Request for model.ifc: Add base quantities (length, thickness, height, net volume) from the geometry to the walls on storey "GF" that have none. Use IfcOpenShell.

First a look at what the model holds.

```python
import ifcopenshell
import ifcopenshell.util.element
import ifcopenshell.util.unit

model = ifcopenshell.open("model.ifc")
print(model.schema)
for unit_type in ("LENGTHUNIT", "AREAUNIT", "VOLUMEUNIT"):
    print(unit_type, ifcopenshell.util.unit.calculate_unit_scale(model, unit_type))
storey = next(s for s in model.by_type("IfcBuildingStorey") if s.Name == "GF")
walls = [e for e in ifcopenshell.util.element.get_decomposition(storey) if e.is_a("IfcWall")]
for e in sorted(walls, key=lambda e: e.id()):
    print(e.id(), e.is_a(), e.Name, list(ifcopenshell.util.element.get_psets(e, qtos_only=True)), sep=" | ")
```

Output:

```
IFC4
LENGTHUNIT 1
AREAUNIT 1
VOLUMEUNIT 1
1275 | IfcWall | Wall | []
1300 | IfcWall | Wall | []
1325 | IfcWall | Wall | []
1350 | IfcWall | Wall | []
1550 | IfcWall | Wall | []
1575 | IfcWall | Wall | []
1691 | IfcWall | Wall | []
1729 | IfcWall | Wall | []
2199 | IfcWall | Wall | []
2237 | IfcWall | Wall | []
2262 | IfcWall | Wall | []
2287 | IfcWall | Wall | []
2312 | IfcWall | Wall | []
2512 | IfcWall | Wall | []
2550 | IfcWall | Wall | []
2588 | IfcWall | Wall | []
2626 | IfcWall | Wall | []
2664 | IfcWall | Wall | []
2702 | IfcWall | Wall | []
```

```python
import ifcopenshell
import ifcopenshell.api.pset
import ifcopenshell.geom
import ifcopenshell.util.element
import ifcopenshell.util.shape
import ifcopenshell.util.unit

model = ifcopenshell.open("model.ifc")
unit_scale = ifcopenshell.util.unit.calculate_unit_scale(model)
volume_scale = ifcopenshell.util.unit.calculate_unit_scale(model, "VOLUMEUNIT")
settings = ifcopenshell.geom.settings()

storey = next(s for s in model.by_type("IfcBuildingStorey") if s.Name == "GF")
walls = [e for e in ifcopenshell.util.element.get_decomposition(storey) if e.is_a("IfcWall")]

for e in sorted(walls, key=lambda e: e.id()):
    if ifcopenshell.util.element.get_psets(e, qtos_only=True, should_inherit=False):
        continue
    # Geometry comes back in metres, in the element's own axes.
    shape = ifcopenshell.geom.create_shape(settings, e)
    values = {
        "Length": ifcopenshell.util.shape.get_x(shape.geometry) / unit_scale,
        "Width": ifcopenshell.util.shape.get_y(shape.geometry) / unit_scale,
        "Height": ifcopenshell.util.shape.get_z(shape.geometry) / unit_scale,
        "NetVolume": ifcopenshell.util.shape.get_volume(shape.geometry) / volume_scale,
    }
    qto = ifcopenshell.api.pset.add_qto(model, product=e, name="Qto_WallBaseQuantities")
    ifcopenshell.api.pset.edit_qto(model, qto=qto, properties=values)
    print(e.id(), {k: round(v, 3) for k, v in values.items()})

model.write("model_rev.ifc")
```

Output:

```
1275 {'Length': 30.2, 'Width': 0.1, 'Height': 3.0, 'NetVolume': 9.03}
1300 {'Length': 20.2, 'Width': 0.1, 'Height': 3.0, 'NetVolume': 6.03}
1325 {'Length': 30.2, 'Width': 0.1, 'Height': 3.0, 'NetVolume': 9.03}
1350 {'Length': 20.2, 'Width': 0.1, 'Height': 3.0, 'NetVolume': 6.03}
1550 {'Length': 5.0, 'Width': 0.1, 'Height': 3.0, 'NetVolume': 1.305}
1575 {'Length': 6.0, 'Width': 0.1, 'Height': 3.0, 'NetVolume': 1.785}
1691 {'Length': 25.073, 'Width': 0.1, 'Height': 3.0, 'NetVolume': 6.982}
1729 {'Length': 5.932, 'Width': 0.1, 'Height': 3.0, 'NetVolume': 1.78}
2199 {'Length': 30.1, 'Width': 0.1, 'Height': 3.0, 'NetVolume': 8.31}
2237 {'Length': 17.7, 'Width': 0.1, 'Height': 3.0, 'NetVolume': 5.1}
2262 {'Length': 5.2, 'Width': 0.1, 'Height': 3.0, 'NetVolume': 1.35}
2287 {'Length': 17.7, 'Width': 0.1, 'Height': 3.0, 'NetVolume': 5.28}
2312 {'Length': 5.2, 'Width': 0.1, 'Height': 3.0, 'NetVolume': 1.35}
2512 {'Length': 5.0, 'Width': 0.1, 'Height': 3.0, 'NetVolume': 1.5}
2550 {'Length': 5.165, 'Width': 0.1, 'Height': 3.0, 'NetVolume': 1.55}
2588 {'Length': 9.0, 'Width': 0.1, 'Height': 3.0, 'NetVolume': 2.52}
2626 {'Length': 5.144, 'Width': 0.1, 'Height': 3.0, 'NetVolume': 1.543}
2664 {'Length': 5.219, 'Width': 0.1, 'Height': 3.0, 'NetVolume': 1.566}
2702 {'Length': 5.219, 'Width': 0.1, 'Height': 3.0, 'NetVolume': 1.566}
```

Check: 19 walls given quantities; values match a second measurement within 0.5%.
